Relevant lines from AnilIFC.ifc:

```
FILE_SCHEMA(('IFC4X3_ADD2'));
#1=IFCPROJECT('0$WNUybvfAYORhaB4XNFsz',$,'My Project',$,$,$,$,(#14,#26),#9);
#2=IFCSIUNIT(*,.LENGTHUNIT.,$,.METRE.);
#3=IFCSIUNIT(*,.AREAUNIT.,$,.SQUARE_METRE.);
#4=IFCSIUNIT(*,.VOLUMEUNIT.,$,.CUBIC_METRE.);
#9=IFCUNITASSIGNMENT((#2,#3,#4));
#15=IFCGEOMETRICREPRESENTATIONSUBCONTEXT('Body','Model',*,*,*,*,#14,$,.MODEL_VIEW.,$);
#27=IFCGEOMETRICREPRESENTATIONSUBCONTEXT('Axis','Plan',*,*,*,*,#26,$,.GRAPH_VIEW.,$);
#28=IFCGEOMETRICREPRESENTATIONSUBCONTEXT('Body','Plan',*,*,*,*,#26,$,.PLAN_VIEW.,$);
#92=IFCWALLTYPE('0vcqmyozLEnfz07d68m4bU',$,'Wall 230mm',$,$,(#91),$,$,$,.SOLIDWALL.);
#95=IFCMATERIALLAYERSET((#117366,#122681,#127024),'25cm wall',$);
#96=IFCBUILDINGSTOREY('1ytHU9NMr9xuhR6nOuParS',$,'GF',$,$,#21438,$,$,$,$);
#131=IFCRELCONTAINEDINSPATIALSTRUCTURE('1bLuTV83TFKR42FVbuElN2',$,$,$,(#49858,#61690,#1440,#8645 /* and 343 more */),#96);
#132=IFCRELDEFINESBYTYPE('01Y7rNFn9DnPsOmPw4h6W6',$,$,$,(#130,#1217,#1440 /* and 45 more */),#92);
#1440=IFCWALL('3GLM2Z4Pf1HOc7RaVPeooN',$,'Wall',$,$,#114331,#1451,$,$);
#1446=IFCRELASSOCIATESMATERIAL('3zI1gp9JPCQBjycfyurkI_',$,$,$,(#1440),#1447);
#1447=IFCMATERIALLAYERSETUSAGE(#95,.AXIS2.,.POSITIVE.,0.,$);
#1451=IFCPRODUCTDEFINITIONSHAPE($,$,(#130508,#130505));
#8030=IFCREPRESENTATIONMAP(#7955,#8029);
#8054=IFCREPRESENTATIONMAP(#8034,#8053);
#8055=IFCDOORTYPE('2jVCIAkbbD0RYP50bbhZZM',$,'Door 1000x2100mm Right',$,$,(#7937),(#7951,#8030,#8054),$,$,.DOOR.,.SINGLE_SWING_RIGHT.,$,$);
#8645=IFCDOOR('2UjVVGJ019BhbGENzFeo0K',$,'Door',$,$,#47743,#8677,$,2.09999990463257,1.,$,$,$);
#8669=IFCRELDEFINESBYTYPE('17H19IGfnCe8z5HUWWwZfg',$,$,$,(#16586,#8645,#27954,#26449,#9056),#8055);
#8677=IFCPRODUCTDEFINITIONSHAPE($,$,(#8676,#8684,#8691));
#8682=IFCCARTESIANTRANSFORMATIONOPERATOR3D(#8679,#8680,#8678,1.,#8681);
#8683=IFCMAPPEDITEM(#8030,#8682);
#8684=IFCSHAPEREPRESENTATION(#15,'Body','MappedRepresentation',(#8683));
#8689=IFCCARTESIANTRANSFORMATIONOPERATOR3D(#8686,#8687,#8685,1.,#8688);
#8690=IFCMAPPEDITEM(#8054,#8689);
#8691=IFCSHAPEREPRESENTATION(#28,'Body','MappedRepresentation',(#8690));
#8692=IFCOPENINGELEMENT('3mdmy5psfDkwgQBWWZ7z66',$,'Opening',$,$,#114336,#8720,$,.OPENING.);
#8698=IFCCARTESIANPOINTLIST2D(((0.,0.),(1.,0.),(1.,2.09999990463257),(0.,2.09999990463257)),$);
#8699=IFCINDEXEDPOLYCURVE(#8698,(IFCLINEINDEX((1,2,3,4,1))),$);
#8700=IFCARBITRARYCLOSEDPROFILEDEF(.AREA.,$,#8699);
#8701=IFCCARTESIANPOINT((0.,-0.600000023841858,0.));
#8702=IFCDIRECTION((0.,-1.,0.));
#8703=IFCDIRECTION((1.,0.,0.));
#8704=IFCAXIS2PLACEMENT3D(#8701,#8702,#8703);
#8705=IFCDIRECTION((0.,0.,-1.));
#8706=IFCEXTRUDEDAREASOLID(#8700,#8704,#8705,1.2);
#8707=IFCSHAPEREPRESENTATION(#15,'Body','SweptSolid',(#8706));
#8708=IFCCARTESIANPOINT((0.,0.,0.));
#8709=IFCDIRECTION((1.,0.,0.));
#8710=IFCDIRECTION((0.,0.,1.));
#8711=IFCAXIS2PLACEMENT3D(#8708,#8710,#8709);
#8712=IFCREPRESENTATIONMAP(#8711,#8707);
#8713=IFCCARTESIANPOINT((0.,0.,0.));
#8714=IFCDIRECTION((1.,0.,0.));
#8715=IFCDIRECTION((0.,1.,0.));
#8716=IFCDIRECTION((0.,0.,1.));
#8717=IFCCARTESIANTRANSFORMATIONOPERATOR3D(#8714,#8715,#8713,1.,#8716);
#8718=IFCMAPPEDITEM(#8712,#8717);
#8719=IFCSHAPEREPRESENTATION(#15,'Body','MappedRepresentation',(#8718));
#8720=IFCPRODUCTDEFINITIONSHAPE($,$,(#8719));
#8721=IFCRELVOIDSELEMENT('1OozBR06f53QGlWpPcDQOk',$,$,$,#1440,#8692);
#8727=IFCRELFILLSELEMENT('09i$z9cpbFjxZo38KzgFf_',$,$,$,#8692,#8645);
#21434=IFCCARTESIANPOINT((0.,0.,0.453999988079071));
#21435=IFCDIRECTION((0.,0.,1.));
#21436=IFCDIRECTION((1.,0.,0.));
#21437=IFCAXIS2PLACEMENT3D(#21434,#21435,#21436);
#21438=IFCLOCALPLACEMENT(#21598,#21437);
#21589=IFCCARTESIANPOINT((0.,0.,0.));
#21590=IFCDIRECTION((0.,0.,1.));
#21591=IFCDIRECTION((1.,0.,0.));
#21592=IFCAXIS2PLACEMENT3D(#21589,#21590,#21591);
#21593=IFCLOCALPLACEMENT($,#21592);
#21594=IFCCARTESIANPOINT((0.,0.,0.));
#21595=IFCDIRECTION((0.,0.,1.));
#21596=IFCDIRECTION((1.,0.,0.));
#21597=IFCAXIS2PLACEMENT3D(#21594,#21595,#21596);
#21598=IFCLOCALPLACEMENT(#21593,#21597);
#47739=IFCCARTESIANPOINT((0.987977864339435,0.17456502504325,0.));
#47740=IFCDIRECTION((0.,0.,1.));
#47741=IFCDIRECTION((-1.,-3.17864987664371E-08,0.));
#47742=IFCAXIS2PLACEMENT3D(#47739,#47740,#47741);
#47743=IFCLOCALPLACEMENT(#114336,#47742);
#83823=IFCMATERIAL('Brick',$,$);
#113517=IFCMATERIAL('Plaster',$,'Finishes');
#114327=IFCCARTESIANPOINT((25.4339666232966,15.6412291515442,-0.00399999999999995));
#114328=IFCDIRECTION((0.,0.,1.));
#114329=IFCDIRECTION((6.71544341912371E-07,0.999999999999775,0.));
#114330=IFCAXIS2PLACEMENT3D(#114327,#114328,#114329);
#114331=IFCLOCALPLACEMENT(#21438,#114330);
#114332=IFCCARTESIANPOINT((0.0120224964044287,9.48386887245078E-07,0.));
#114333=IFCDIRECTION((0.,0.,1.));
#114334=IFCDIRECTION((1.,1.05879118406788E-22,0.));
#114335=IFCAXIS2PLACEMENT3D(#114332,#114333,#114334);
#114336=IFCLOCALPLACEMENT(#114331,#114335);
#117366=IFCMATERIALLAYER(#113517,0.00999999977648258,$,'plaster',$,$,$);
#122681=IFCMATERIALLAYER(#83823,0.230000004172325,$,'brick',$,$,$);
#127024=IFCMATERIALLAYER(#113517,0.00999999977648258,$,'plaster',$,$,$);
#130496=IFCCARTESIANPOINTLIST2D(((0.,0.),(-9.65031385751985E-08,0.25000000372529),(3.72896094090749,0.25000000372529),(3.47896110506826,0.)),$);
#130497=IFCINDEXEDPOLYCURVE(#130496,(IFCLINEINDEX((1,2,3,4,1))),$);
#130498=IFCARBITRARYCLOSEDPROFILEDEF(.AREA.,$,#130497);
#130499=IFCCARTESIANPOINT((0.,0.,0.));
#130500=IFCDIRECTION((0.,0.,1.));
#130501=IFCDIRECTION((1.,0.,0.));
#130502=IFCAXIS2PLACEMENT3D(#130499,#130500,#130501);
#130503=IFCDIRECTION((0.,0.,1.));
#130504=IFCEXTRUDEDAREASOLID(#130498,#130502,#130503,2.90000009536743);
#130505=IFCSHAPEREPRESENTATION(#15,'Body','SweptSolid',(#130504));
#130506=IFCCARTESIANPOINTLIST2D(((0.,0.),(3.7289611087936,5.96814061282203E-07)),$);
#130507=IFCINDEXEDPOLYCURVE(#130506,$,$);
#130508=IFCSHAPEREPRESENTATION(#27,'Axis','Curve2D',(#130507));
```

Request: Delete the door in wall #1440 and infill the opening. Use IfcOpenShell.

```python
import ifcopenshell
import ifcopenshell.api.feature
import ifcopenshell.api.root
import ifcopenshell.geom
import ifcopenshell.util.shape

model = ifcopenshell.open("AnilIFC.ifc")
settings = ifcopenshell.geom.settings()


def volume(element):
    """Net volume in cubic metres, openings subtracted."""
    shape = ifcopenshell.geom.create_shape(settings, element)
    return ifcopenshell.util.shape.get_volume(shape.geometry)


door = model.by_guid("2UjVVGJ019BhbGENzFeo0K")
opening = door.FillsVoids[0].RelatingOpeningElement
wall = opening.VoidsElements[0].RelatingBuildingElement
before = volume(wall)

ifcopenshell.api.root.remove_product(model, product=door)
ifcopenshell.api.feature.remove_feature(model, feature=opening)

after = volume(wall)

print(f"wall volume {before:.3f} -> {after:.3f} m3")

model.write("AnilIFC_edited.ifc")
```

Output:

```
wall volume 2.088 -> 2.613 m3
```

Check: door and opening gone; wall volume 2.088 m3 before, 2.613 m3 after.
